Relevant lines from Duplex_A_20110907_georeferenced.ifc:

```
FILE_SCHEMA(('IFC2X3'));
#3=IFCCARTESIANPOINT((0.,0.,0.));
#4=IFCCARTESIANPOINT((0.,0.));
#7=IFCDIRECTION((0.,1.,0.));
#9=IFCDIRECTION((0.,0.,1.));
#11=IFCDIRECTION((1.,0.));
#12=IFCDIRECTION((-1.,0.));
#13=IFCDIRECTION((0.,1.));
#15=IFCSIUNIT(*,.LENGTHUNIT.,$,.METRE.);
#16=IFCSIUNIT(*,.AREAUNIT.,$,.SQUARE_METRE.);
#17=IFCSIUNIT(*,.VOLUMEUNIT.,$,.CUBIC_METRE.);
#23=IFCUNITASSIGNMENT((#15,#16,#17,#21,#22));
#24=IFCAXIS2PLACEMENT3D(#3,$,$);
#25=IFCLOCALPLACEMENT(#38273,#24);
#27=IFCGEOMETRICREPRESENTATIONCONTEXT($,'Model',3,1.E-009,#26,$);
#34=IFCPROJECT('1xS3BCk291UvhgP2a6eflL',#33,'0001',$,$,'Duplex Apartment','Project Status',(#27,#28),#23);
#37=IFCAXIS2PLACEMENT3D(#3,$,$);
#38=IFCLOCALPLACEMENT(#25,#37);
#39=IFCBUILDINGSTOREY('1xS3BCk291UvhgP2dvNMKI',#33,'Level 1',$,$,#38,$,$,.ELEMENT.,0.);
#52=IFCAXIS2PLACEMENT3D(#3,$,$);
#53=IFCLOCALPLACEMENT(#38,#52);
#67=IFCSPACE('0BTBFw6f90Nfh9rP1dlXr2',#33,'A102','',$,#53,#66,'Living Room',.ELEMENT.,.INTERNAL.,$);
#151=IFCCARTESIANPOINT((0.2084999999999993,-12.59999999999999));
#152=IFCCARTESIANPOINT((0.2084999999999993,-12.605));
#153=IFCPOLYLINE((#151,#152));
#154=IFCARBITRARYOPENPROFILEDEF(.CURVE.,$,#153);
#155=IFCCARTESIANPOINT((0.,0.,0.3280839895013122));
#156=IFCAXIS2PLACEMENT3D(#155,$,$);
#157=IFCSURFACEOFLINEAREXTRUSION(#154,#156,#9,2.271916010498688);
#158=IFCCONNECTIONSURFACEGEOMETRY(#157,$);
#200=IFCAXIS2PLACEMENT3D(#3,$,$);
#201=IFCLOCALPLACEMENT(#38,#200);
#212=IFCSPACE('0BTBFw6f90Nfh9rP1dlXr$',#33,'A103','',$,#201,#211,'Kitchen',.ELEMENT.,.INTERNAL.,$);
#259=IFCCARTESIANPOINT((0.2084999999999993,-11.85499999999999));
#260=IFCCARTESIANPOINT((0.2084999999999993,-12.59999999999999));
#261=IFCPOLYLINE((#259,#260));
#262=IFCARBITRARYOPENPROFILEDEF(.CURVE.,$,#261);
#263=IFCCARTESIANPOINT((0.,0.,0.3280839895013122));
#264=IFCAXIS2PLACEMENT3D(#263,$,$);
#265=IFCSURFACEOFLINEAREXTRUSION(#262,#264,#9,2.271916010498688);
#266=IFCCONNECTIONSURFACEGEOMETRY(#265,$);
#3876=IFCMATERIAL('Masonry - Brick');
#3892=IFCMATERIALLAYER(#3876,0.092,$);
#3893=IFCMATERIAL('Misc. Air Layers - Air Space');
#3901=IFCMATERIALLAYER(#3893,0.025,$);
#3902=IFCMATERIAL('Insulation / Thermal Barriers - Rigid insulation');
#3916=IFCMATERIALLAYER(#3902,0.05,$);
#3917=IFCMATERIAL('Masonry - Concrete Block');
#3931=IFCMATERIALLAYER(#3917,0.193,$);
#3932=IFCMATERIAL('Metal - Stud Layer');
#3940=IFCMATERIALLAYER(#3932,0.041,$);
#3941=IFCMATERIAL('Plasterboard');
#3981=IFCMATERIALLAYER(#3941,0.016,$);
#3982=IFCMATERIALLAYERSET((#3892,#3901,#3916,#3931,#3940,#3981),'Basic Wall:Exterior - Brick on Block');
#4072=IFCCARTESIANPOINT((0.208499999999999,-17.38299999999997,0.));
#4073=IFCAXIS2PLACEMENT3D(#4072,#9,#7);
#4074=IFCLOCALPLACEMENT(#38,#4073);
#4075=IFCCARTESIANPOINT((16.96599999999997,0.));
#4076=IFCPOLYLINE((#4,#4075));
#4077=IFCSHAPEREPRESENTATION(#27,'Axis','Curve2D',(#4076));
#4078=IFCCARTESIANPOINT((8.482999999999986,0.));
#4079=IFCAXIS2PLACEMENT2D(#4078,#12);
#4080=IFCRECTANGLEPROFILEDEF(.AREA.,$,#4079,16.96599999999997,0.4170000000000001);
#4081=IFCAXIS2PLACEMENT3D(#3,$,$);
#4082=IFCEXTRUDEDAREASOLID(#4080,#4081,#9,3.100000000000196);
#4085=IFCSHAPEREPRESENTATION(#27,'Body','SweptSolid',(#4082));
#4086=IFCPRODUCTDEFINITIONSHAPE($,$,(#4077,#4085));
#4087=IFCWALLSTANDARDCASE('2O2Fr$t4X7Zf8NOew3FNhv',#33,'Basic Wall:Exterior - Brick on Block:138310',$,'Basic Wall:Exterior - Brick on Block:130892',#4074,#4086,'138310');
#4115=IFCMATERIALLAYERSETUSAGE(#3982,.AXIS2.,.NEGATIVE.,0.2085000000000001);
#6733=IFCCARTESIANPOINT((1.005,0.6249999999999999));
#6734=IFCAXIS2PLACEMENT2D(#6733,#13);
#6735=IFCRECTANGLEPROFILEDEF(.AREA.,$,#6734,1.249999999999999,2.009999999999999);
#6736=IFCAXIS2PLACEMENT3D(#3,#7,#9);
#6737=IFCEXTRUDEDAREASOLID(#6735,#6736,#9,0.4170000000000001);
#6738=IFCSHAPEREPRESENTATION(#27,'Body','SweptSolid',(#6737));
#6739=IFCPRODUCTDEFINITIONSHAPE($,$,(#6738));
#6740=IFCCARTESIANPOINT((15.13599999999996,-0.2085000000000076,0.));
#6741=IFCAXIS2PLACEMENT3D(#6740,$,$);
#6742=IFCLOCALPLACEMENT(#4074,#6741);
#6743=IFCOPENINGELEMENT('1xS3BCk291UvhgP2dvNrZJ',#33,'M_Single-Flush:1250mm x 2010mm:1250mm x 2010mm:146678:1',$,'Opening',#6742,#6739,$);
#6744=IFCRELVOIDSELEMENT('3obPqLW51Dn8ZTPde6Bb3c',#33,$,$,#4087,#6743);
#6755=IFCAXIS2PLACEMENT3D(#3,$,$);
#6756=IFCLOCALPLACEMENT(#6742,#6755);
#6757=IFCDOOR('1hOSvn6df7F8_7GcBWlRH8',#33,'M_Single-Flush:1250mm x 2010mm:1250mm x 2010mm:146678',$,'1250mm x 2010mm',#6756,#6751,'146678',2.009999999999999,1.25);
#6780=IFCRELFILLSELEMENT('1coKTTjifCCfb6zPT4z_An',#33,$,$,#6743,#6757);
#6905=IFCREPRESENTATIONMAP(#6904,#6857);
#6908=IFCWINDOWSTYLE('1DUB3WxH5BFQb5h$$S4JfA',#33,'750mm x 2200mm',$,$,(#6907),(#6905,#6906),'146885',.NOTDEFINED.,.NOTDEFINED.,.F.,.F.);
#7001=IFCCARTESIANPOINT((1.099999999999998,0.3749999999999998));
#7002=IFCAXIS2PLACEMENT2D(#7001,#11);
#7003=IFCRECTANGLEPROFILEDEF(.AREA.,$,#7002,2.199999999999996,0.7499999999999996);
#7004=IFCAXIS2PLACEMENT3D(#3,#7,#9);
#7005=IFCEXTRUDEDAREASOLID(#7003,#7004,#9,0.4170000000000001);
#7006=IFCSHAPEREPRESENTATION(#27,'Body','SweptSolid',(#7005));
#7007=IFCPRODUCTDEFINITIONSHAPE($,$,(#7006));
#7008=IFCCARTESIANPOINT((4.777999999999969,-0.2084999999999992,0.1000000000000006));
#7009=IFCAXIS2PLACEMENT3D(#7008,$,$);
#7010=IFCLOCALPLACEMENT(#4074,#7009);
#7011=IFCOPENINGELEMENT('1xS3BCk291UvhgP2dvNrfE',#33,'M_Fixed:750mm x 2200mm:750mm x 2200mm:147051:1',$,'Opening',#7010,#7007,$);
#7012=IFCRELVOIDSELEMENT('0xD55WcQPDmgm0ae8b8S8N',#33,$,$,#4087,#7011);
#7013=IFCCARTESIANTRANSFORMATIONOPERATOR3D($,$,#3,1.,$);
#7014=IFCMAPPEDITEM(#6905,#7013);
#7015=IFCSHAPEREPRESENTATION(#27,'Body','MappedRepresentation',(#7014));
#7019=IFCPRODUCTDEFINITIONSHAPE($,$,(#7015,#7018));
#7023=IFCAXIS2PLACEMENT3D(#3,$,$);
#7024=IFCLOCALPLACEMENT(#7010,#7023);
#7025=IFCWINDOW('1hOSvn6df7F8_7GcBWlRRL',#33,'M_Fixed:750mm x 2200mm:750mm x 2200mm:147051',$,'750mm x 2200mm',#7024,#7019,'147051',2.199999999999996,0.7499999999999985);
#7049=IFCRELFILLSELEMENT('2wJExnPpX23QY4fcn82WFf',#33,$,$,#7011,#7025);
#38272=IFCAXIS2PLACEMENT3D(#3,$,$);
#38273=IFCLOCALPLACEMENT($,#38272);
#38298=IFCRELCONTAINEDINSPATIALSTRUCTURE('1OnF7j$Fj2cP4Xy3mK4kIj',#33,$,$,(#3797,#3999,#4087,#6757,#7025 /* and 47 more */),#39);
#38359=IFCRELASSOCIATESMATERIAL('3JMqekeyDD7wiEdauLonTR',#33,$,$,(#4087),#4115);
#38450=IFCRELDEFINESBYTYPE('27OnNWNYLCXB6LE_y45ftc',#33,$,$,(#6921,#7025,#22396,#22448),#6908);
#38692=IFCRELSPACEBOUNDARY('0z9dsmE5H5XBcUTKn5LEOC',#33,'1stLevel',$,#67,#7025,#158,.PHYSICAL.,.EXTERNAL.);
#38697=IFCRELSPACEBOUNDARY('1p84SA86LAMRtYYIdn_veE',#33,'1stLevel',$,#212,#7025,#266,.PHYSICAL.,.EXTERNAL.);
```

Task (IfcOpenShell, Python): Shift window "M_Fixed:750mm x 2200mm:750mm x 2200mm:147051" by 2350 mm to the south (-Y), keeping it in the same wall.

```python
import numpy as np
import ifcopenshell
import ifcopenshell.api.geometry
import ifcopenshell.util.placement

model = ifcopenshell.open("Duplex_A_20110907_georeferenced.ifc")

window = model.by_id(7025)
opening = window.FillsVoids[0].RelatingOpeningElement
wall = opening.VoidsElements[0].RelatingBuildingElement

wall_matrix = ifcopenshell.util.placement.get_local_placement(wall.ObjectPlacement)
shift = wall_matrix[:3, 0] * -2.35
before = ifcopenshell.util.placement.get_local_placement(window.ObjectPlacement)[:3, 3].copy()

# The window is placed relative to its opening, so it follows when the opening moves.
matrix = ifcopenshell.util.placement.get_local_placement(opening.ObjectPlacement)
matrix[:3, 3] += shift
ifcopenshell.api.geometry.edit_object_placement(
    model, product=opening, matrix=matrix, is_si=False, should_transform_children=True
)

# Space boundary surfaces are stored in each space's coordinates; move them too.
for rel in window.ProvidesBoundaries:
    if not rel.ConnectionGeometry:
        continue
    surface = rel.ConnectionGeometry.SurfaceOnRelatingElement
    space_matrix = ifcopenshell.util.placement.get_local_placement(rel.RelatingSpace.ObjectPlacement)
    point = np.array(surface.Position.Location.Coordinates) + space_matrix[:3, :3].T @ shift
    surface.Position = model.createIfcAxis2Placement3D(
        model.createIfcCartesianPoint(point.tolist()), surface.Position.Axis, surface.Position.RefDirection
    )

after = ifcopenshell.util.placement.get_local_placement(window.ObjectPlacement)[:3, 3]
print("window moved by", (after - before).round(3) + 0.0)

model.write("Duplex_A_20110907_georeferenced_v2.ifc")
```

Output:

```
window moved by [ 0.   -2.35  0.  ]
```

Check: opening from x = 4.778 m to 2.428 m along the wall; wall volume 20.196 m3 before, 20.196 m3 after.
